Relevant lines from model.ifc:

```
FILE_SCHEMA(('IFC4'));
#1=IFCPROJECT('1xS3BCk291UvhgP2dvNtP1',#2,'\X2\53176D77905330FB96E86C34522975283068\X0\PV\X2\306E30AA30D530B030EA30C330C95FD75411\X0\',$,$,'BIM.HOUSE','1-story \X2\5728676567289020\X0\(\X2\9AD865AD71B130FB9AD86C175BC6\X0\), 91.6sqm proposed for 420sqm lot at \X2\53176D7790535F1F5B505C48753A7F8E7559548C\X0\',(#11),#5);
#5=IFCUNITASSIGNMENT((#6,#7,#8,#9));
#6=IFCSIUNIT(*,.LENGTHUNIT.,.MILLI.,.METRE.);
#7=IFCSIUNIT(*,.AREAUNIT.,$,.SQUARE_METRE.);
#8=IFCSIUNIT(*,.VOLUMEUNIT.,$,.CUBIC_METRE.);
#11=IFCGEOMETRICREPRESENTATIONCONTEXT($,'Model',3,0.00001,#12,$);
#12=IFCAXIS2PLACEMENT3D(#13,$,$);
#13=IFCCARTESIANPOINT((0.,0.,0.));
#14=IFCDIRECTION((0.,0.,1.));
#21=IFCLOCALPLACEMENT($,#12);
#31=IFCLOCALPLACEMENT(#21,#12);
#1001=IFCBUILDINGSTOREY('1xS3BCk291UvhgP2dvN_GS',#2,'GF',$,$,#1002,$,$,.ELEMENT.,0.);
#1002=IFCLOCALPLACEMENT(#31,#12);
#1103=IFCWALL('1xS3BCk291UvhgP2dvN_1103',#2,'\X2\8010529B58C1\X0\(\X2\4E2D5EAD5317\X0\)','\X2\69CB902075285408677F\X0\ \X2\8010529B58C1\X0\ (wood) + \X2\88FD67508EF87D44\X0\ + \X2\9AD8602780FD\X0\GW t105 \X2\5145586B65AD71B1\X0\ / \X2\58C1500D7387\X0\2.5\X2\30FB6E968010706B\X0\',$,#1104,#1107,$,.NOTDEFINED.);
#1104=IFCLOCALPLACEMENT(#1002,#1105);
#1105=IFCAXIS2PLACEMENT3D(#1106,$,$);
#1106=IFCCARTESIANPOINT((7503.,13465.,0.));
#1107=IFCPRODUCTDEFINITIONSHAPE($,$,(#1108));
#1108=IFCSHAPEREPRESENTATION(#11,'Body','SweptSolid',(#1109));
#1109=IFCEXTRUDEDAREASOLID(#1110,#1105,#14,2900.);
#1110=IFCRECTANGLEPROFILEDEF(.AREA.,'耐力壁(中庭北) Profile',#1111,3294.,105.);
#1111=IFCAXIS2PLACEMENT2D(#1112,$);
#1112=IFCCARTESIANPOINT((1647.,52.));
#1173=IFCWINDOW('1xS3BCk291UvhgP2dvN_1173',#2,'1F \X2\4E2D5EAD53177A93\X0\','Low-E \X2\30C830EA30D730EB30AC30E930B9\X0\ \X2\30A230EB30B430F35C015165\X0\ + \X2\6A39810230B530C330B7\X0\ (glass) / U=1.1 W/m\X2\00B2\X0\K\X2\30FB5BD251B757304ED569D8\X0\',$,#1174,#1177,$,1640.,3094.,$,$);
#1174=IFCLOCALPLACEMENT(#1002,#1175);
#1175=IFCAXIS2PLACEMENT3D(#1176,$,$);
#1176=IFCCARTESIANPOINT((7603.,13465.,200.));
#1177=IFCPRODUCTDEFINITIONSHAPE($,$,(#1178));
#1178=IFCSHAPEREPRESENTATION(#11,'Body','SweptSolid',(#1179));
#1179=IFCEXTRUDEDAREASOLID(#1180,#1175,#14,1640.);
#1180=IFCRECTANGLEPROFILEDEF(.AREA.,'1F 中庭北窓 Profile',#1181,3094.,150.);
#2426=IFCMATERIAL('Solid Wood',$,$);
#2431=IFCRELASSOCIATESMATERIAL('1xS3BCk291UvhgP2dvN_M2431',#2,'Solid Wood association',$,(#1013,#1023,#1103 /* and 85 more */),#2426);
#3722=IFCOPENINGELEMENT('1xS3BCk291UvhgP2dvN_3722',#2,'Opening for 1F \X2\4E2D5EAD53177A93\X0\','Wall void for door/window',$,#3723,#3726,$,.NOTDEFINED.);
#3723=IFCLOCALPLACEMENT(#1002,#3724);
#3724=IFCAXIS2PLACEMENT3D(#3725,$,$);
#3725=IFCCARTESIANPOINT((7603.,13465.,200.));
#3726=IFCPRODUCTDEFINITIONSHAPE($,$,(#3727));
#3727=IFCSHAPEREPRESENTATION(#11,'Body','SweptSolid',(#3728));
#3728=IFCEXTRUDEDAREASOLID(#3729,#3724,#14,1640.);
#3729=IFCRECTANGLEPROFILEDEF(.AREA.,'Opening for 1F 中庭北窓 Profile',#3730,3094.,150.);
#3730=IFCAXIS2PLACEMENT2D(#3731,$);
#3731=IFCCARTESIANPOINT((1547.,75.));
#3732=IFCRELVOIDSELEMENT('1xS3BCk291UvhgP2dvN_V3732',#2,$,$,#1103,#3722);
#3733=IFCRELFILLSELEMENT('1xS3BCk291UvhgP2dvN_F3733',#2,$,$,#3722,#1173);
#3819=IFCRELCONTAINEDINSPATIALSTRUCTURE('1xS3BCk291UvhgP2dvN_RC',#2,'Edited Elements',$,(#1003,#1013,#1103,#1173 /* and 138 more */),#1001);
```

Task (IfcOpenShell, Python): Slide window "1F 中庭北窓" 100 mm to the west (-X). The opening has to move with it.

```python
import ifcopenshell
import ifcopenshell.api.geometry
import ifcopenshell.util.placement
import ifcopenshell.util.unit

model = ifcopenshell.open("model.ifc")
unit_scale = ifcopenshell.util.unit.calculate_unit_scale(model)

window = model.by_guid("1xS3BCk291UvhgP2dvN_1173")
opening = window.FillsVoids[0].RelatingOpeningElement
wall = opening.VoidsElements[0].RelatingBuildingElement

wall_matrix = ifcopenshell.util.placement.get_local_placement(wall.ObjectPlacement)
shift = wall_matrix[:3, 0] * -0.1 / unit_scale
before = ifcopenshell.util.placement.get_local_placement(window.ObjectPlacement)[:3, 3].copy()

# The window is not placed relative to its opening, so move both.
for product in (opening, window):
    matrix = ifcopenshell.util.placement.get_local_placement(product.ObjectPlacement)
    matrix[:3, 3] += shift
    ifcopenshell.api.geometry.edit_object_placement(model, product=product, matrix=matrix, is_si=False)

after = ifcopenshell.util.placement.get_local_placement(window.ObjectPlacement)[:3, 3]
print("window moved by", (after - before).round(3) + 0.0)

model.write("model_edited.ifc")
```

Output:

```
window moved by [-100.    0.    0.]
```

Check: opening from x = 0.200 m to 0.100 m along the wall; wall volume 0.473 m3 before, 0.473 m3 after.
